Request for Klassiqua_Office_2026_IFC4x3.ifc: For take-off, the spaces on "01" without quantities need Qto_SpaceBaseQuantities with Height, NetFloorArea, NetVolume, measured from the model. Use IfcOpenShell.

First a look at what the model holds.

```python
import ifcopenshell
import ifcopenshell.util.element
import ifcopenshell.util.unit

model = ifcopenshell.open("Klassiqua_Office_2026_IFC4x3.ifc")
print(model.schema)
for unit_type in ("LENGTHUNIT", "AREAUNIT", "VOLUMEUNIT"):
    print(unit_type, ifcopenshell.util.unit.calculate_unit_scale(model, unit_type))
storey = next(s for s in model.by_type("IfcBuildingStorey") if s.Name == "01")
spaces = [e for e in ifcopenshell.util.element.get_decomposition(storey) if e.is_a("IfcSpace")]
for e in sorted(spaces, key=lambda e: e.id()):
    print(e.id(), e.is_a(), e.Name, list(ifcopenshell.util.element.get_psets(e, qtos_only=True)), sep=" | ")
```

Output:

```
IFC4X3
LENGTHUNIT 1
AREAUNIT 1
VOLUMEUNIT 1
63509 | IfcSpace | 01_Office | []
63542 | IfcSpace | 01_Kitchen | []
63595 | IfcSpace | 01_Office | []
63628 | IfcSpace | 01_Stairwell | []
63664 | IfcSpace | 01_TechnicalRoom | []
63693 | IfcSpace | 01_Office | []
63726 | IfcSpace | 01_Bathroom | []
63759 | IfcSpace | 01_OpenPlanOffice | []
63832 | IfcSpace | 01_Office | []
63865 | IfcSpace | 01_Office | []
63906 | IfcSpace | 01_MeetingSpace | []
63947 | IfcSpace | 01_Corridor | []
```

```python
import ifcopenshell
import ifcopenshell.api.pset
import ifcopenshell.geom
import ifcopenshell.util.element
import ifcopenshell.util.shape
import ifcopenshell.util.unit

model = ifcopenshell.open("Klassiqua_Office_2026_IFC4x3.ifc")
unit_scale = ifcopenshell.util.unit.calculate_unit_scale(model)
area_scale = ifcopenshell.util.unit.calculate_unit_scale(model, "AREAUNIT")
volume_scale = ifcopenshell.util.unit.calculate_unit_scale(model, "VOLUMEUNIT")
settings = ifcopenshell.geom.settings()

storey = next(s for s in model.by_type("IfcBuildingStorey") if s.Name == "01")
spaces = [e for e in ifcopenshell.util.element.get_decomposition(storey) if e.is_a("IfcSpace")]

for e in sorted(spaces, key=lambda e: e.id()):
    if ifcopenshell.util.element.get_psets(e, qtos_only=True, should_inherit=False):
        continue
    # Geometry comes back in metres, in the element's own axes.
    shape = ifcopenshell.geom.create_shape(settings, e)
    values = {
        "Height": ifcopenshell.util.shape.get_z(shape.geometry) / unit_scale,
        "NetFloorArea": ifcopenshell.util.shape.get_footprint_area(shape.geometry) / area_scale,
        "NetVolume": ifcopenshell.util.shape.get_volume(shape.geometry) / volume_scale,
    }
    qto = ifcopenshell.api.pset.add_qto(model, product=e, name="Qto_SpaceBaseQuantities")
    ifcopenshell.api.pset.edit_qto(model, qto=qto, properties=values)
    print(e.id(), {k: round(v, 3) for k, v in values.items()})

model.write("Klassiqua_Office_2026_IFC4x3_updated.ifc")
```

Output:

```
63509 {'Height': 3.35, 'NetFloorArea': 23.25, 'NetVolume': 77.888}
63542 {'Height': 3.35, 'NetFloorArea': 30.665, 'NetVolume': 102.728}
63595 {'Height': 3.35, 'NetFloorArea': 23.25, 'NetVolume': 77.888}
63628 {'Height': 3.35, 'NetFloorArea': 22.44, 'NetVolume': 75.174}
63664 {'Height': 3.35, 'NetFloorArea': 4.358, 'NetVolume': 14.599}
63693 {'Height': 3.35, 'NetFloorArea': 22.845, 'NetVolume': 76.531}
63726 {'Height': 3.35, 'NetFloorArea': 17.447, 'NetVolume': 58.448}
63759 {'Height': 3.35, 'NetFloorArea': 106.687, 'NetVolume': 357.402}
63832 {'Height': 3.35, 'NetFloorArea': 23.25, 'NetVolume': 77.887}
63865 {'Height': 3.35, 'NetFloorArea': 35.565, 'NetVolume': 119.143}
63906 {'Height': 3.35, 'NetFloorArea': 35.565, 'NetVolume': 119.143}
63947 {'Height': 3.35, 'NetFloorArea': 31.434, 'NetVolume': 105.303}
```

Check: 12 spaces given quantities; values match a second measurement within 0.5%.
